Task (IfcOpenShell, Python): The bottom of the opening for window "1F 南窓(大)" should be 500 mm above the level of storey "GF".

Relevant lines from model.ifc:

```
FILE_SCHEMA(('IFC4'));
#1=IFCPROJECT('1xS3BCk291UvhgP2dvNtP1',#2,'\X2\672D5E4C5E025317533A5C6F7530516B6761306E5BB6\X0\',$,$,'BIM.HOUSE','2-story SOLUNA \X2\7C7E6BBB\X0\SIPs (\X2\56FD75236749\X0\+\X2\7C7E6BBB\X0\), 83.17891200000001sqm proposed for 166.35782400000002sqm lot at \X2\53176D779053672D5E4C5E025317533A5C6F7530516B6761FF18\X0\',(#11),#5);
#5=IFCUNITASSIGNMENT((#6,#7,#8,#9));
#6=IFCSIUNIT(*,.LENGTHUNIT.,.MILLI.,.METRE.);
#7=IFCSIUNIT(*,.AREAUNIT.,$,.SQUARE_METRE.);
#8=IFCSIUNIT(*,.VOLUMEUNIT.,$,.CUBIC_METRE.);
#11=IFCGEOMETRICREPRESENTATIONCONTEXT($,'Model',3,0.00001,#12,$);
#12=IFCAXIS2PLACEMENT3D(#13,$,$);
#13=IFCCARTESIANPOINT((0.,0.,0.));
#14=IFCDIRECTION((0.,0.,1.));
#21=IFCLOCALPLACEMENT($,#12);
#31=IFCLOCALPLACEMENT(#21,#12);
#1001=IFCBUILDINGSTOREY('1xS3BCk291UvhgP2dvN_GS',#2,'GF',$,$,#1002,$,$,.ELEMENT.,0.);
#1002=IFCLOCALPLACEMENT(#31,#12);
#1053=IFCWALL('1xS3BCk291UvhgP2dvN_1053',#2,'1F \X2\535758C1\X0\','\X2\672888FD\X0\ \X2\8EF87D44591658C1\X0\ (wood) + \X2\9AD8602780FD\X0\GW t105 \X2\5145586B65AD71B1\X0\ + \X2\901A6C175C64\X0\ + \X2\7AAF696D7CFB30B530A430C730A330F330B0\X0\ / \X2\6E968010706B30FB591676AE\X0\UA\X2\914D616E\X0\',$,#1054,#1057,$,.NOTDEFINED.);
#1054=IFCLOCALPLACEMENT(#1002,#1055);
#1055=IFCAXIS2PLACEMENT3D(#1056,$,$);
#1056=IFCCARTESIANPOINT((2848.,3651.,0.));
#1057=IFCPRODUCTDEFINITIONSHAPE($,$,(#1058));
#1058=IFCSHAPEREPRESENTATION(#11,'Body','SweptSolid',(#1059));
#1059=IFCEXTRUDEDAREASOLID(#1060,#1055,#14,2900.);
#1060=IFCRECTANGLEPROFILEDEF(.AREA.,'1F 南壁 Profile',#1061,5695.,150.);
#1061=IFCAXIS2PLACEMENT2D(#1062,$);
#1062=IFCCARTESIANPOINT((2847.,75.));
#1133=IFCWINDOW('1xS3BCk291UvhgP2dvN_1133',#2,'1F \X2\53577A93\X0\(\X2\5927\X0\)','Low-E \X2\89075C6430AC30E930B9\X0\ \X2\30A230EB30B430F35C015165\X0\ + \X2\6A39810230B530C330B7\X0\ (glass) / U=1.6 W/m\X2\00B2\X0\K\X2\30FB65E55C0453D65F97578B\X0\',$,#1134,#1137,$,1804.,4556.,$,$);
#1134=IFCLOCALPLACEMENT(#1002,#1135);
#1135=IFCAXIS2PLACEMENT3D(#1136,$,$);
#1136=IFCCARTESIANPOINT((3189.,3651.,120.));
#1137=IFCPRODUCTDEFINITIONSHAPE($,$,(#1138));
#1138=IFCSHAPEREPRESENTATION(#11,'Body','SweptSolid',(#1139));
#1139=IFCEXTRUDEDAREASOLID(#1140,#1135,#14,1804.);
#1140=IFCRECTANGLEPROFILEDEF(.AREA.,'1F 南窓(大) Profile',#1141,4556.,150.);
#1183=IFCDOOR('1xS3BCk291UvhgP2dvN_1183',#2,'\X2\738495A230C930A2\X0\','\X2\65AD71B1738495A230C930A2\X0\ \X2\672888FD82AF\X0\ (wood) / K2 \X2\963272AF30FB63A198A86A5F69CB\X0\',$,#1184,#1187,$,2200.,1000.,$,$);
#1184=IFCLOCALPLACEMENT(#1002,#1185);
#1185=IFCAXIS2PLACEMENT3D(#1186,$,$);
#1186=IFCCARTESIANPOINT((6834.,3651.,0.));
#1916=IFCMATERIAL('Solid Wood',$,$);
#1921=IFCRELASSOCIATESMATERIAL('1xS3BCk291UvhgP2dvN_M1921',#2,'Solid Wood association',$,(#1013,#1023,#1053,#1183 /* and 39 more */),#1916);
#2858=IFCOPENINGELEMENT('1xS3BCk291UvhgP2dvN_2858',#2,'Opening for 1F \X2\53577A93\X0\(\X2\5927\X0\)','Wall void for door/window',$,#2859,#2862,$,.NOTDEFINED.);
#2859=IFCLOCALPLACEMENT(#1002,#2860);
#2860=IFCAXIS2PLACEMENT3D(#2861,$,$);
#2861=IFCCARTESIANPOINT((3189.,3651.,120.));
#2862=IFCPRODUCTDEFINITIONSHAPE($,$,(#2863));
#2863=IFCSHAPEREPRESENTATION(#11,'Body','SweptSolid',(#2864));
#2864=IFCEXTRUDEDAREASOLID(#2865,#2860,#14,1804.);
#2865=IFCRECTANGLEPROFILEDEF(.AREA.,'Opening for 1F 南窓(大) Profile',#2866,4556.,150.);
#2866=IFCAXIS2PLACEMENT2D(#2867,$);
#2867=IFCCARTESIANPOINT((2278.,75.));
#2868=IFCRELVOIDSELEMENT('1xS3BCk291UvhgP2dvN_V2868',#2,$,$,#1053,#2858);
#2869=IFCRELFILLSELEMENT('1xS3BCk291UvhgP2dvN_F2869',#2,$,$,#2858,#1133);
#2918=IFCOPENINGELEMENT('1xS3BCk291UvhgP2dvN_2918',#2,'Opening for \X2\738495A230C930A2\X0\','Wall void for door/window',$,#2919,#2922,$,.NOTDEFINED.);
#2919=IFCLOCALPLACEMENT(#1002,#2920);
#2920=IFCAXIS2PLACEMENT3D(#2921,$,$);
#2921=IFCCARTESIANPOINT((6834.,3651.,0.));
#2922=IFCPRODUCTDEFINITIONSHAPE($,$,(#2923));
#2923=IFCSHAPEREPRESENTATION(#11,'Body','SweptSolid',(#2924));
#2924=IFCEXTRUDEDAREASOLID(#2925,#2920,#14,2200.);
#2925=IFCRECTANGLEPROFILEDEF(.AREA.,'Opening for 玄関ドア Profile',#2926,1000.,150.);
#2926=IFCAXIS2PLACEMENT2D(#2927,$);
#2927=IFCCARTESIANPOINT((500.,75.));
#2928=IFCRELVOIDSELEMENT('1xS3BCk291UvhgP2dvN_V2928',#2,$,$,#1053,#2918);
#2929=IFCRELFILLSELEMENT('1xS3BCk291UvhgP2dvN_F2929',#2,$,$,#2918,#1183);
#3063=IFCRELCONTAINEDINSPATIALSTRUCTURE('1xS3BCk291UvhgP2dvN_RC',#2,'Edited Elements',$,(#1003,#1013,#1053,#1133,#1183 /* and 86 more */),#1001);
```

```python
import numpy as np
import ifcopenshell
import ifcopenshell.api.geometry
import ifcopenshell.geom
import ifcopenshell.util.element
import ifcopenshell.util.placement
import ifcopenshell.util.shape
import ifcopenshell.util.unit

model = ifcopenshell.open("model.ifc")
unit_scale = ifcopenshell.util.unit.calculate_unit_scale(model)

window = model.by_guid("1xS3BCk291UvhgP2dvN_1133")
opening = window.FillsVoids[0].RelatingOpeningElement
storey = ifcopenshell.util.element.get_container(window, ifc_class="IfcBuildingStorey")
level = ifcopenshell.util.placement.get_local_placement(storey.ObjectPlacement)[2, 3]

# The opening's origin need not be at the sill, so measure its lowest point.
shape = ifcopenshell.geom.create_shape(ifcopenshell.geom.settings(), opening)
bottom = ifcopenshell.util.shape.get_shape_bottom_elevation(shape, shape.geometry) / unit_scale
dz = level + 0.5 / unit_scale - bottom

shift = np.array([0.0, 0.0, dz])
# The window is not placed relative to its opening, so move both.
for product in (opening, window):
    matrix = ifcopenshell.util.placement.get_local_placement(product.ObjectPlacement)
    matrix[:3, 3] += shift
    ifcopenshell.api.geometry.edit_object_placement(model, product=product, matrix=matrix, is_si=False)

print(f"moved by {dz * unit_scale:+.3f} m")

model.write("model_v2.ifc")
```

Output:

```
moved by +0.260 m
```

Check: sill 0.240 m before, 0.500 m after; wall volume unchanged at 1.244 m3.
